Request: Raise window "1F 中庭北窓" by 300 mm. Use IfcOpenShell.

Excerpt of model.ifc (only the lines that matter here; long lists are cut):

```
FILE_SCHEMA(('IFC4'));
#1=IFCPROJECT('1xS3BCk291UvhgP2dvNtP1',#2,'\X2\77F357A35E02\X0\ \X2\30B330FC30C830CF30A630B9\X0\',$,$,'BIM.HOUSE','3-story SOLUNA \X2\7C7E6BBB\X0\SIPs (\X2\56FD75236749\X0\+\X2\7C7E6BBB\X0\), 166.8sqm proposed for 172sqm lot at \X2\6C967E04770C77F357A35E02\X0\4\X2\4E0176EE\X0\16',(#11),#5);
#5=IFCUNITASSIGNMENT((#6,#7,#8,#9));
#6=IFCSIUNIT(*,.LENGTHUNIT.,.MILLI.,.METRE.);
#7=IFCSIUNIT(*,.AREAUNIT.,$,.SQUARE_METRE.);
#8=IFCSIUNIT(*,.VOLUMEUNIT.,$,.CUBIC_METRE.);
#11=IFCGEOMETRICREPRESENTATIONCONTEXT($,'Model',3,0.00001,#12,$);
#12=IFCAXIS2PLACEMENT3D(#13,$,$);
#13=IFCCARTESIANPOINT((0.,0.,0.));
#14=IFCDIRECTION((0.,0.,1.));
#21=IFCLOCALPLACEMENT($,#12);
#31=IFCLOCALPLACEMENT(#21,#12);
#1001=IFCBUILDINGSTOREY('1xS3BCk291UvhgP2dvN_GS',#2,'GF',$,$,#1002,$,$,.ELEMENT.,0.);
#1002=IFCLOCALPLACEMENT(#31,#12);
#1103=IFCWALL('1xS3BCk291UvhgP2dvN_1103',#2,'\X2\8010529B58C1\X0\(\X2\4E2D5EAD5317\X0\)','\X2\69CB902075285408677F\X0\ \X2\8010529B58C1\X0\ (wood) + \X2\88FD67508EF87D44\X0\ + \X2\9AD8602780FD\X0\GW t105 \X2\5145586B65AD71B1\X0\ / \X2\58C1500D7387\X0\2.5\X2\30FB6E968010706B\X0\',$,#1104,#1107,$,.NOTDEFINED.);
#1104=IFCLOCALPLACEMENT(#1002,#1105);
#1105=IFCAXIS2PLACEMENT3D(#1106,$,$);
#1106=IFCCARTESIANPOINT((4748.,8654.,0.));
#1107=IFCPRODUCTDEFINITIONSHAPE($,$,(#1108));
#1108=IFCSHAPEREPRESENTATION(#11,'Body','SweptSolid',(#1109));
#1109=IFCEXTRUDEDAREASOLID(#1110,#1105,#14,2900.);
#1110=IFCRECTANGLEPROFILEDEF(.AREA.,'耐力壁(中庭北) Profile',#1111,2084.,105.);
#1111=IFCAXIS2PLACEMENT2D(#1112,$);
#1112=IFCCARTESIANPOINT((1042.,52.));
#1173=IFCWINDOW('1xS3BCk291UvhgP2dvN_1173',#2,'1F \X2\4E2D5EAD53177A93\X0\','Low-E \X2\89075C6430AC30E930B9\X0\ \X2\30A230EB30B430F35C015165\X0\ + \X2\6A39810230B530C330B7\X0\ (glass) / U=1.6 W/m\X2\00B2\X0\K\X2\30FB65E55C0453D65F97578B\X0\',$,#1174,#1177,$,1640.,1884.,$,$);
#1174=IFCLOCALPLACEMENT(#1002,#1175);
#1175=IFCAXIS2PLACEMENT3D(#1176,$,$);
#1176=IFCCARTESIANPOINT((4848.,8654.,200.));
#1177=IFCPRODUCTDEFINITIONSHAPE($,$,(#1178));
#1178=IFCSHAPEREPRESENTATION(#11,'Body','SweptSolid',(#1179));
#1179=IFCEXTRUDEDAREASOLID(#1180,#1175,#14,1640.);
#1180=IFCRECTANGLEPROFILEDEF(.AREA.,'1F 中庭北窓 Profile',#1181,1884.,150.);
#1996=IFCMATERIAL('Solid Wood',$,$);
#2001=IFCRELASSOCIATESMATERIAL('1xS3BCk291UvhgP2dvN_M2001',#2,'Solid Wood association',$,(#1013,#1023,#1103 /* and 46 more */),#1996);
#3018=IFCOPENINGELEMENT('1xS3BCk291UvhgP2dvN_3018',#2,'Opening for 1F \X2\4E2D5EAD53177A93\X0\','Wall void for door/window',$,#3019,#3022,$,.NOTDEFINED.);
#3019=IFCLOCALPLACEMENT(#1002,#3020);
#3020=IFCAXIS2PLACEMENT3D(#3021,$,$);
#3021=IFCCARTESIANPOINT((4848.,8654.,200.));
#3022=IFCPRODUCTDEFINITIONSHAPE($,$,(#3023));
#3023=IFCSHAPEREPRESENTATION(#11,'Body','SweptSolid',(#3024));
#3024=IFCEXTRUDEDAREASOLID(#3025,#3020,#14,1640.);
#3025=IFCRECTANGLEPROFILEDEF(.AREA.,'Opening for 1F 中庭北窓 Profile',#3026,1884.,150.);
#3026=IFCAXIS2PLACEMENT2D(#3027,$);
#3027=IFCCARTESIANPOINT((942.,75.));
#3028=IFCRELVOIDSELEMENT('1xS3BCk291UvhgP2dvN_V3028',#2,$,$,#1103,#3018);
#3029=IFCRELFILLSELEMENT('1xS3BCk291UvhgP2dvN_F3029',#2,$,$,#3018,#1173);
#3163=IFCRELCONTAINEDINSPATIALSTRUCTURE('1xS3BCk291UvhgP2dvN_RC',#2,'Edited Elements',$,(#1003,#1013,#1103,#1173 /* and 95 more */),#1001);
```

```python
import numpy as np
import ifcopenshell
import ifcopenshell.api.geometry
import ifcopenshell.util.placement
import ifcopenshell.util.unit

model = ifcopenshell.open("model.ifc")
unit_scale = ifcopenshell.util.unit.calculate_unit_scale(model)

window = model.by_guid("1xS3BCk291UvhgP2dvN_1173")
opening = window.FillsVoids[0].RelatingOpeningElement
dz = 0.3 / unit_scale

shift = np.array([0.0, 0.0, dz])
# The window is not placed relative to its opening, so move both.
for product in (opening, window):
    matrix = ifcopenshell.util.placement.get_local_placement(product.ObjectPlacement)
    matrix[:3, 3] += shift
    ifcopenshell.api.geometry.edit_object_placement(model, product=product, matrix=matrix, is_si=False)

print(f"moved by {dz * unit_scale:+.3f} m")

model.write("model_edited.ifc")
```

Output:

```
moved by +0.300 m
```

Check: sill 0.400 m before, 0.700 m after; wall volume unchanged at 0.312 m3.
